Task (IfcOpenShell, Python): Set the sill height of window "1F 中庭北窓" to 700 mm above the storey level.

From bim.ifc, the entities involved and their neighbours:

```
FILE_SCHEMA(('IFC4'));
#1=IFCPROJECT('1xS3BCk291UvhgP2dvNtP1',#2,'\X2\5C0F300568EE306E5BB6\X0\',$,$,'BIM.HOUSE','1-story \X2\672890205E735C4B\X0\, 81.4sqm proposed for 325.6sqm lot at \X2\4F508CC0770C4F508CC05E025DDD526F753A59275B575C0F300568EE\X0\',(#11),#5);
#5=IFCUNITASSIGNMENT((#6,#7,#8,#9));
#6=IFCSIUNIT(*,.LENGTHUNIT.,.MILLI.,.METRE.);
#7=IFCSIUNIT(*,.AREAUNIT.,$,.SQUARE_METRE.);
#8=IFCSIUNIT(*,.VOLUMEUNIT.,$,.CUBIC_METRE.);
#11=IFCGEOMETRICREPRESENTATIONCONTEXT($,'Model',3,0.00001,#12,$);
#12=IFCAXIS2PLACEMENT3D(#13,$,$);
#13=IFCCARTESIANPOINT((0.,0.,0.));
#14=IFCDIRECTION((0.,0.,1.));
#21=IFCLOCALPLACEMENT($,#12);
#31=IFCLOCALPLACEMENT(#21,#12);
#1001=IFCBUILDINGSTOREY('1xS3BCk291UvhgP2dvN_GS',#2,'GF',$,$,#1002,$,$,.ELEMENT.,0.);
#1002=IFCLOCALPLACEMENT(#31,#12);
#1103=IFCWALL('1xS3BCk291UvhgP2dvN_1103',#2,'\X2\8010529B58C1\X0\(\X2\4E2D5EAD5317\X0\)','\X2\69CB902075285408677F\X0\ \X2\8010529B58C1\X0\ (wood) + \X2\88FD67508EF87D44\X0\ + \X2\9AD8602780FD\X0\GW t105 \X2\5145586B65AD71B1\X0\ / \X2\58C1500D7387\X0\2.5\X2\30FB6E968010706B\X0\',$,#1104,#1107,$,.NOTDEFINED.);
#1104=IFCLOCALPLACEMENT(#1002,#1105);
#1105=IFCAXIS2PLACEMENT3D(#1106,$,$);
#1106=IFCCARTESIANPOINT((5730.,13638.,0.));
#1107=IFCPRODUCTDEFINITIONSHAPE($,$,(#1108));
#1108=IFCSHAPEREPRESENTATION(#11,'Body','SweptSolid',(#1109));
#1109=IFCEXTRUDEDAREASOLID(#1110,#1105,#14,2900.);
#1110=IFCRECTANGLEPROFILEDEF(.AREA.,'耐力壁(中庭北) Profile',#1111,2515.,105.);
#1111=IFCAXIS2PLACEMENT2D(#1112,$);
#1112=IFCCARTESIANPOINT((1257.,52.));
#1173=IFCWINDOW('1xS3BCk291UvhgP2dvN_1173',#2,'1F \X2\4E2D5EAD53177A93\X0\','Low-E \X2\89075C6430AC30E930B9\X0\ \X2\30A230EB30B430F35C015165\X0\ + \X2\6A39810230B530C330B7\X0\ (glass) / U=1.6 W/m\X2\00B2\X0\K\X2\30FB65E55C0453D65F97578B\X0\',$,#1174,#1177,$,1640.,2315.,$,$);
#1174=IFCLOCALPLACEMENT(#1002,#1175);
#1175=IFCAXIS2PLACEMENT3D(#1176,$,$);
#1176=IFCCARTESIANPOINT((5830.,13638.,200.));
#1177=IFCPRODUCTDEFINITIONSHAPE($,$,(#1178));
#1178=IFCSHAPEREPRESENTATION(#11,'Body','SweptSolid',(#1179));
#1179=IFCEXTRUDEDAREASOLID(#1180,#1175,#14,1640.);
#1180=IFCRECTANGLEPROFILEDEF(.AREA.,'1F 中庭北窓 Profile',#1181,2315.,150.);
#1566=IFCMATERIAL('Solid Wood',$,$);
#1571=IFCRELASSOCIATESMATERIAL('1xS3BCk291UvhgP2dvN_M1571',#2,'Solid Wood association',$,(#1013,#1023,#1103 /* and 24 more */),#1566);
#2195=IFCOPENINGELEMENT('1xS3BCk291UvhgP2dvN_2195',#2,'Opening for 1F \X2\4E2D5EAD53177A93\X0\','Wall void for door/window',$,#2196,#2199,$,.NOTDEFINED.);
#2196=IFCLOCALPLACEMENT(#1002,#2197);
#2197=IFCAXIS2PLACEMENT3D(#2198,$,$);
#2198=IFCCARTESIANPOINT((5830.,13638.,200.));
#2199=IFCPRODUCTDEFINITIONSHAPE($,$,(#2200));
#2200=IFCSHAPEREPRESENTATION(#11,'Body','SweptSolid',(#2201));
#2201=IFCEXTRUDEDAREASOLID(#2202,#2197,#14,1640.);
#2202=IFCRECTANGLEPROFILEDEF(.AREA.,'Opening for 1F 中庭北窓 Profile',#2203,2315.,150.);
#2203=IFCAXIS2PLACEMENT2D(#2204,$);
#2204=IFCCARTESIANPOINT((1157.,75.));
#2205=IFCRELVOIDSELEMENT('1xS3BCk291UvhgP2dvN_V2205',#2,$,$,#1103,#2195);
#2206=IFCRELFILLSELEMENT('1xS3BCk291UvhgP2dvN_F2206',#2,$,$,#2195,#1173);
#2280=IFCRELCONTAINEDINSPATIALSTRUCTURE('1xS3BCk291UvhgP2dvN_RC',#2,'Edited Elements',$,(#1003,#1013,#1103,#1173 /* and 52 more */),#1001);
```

```python
import numpy as np
import ifcopenshell
import ifcopenshell.api.geometry
import ifcopenshell.geom
import ifcopenshell.util.element
import ifcopenshell.util.placement
import ifcopenshell.util.shape
import ifcopenshell.util.unit

model = ifcopenshell.open("bim.ifc")
unit_scale = ifcopenshell.util.unit.calculate_unit_scale(model)

window = model.by_guid("1xS3BCk291UvhgP2dvN_1173")
opening = window.FillsVoids[0].RelatingOpeningElement
storey = ifcopenshell.util.element.get_container(window, ifc_class="IfcBuildingStorey")
level = ifcopenshell.util.placement.get_local_placement(storey.ObjectPlacement)[2, 3]

# The opening's origin need not be at the sill, so measure its lowest point.
shape = ifcopenshell.geom.create_shape(ifcopenshell.geom.settings(), opening)
bottom = ifcopenshell.util.shape.get_shape_bottom_elevation(shape, shape.geometry) / unit_scale
dz = level + 700.0 - bottom

shift = np.array([0.0, 0.0, dz])
# The window is not placed relative to its opening, so move both.
for product in (opening, window):
    matrix = ifcopenshell.util.placement.get_local_placement(product.ObjectPlacement)
    matrix[:3, 3] += shift
    ifcopenshell.api.geometry.edit_object_placement(model, product=product, matrix=matrix, is_si=False)

print(f"moved by {dz * unit_scale:+.3f} m")

model.write("bim_v2.ifc")
```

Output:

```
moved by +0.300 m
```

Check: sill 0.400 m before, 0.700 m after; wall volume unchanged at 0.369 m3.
